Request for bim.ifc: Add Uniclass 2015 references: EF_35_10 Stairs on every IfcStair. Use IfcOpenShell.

First a look at what the model holds.

```python
import ifcopenshell

model = ifcopenshell.open("bim.ifc")
print(model.schema)
print("classifications:", [c.Name for c in model.by_type("IfcClassification")])
for ifc_class in ("IfcDoor", "IfcRoof", "IfcStair", "IfcWall", "IfcWindow"):
    print(ifc_class, len(model.by_type(ifc_class)))
```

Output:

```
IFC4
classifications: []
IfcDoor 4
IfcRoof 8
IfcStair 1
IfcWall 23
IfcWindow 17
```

```python
import ifcopenshell
import ifcopenshell.api.classification

model = ifcopenshell.open("bim.ifc")

system = ifcopenshell.api.classification.add_classification(model, classification="Uniclass 2015")

codes = {
    "IfcStair": ("EF_35_10", "Stairs"),
}
for ifc_class, (code, name) in codes.items():
    products = model.by_type(ifc_class)
    ifcopenshell.api.classification.add_reference(
        model, products=products, classification=system, identification=code, name=name
    )
    print(code, len(products))

model.write("bim-out.ifc")
```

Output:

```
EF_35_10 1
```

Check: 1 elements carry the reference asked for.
